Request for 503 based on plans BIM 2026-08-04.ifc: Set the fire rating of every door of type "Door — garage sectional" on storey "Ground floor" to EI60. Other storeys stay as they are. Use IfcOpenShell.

First a look at what the model holds.

```python
import ifcopenshell
import ifcopenshell.util.element

model = ifcopenshell.open("503 based on plans BIM 2026-08-04.ifc")
print(model.schema)
storey = next(s for s in model.by_type("IfcBuildingStorey") if s.Name == "Ground floor")
doors = [e for e in ifcopenshell.util.element.get_decomposition(storey) if e.is_a("IfcDoor")]
seen = {}
for e in doors:
    element_type = ifcopenshell.util.element.get_type(e)
    key = (element_type.Name if element_type != e and element_type else None, ifcopenshell.util.element.get_pset(e, "Pset_DoorCommon", "FireRating"))
    seen[key] = seen.get(key, 0) + 1
for (name, value), count in sorted(seen.items(), key=str):
    print(count, "x", name, "|", value)
```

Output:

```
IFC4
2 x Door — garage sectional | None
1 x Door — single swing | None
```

```python
import ifcopenshell
import ifcopenshell.api.pset
import ifcopenshell.util.element

model = ifcopenshell.open("503 based on plans BIM 2026-08-04.ifc")

storey = next(s for s in model.by_type("IfcBuildingStorey") if s.Name == "Ground floor")
doors = [e for e in ifcopenshell.util.element.get_decomposition(storey) if e.is_a("IfcDoor")]

count = 0
for e in doors:
    element_type = ifcopenshell.util.element.get_type(e)
    if element_type in (None, e) or element_type.Name != "Door — garage sectional":
        continue
    # add_pset returns the element's existing set when there is one.
    pset = ifcopenshell.api.pset.add_pset(model, product=e, name="Pset_DoorCommon")
    ifcopenshell.api.pset.edit_pset(model, pset=pset, properties={"FireRating": "EI60"})
    count += 1

print(count, "doors updated")

model.write("503 based on plans BIM 2026-08-04_rev.ifc")
```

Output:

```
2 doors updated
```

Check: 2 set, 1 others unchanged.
